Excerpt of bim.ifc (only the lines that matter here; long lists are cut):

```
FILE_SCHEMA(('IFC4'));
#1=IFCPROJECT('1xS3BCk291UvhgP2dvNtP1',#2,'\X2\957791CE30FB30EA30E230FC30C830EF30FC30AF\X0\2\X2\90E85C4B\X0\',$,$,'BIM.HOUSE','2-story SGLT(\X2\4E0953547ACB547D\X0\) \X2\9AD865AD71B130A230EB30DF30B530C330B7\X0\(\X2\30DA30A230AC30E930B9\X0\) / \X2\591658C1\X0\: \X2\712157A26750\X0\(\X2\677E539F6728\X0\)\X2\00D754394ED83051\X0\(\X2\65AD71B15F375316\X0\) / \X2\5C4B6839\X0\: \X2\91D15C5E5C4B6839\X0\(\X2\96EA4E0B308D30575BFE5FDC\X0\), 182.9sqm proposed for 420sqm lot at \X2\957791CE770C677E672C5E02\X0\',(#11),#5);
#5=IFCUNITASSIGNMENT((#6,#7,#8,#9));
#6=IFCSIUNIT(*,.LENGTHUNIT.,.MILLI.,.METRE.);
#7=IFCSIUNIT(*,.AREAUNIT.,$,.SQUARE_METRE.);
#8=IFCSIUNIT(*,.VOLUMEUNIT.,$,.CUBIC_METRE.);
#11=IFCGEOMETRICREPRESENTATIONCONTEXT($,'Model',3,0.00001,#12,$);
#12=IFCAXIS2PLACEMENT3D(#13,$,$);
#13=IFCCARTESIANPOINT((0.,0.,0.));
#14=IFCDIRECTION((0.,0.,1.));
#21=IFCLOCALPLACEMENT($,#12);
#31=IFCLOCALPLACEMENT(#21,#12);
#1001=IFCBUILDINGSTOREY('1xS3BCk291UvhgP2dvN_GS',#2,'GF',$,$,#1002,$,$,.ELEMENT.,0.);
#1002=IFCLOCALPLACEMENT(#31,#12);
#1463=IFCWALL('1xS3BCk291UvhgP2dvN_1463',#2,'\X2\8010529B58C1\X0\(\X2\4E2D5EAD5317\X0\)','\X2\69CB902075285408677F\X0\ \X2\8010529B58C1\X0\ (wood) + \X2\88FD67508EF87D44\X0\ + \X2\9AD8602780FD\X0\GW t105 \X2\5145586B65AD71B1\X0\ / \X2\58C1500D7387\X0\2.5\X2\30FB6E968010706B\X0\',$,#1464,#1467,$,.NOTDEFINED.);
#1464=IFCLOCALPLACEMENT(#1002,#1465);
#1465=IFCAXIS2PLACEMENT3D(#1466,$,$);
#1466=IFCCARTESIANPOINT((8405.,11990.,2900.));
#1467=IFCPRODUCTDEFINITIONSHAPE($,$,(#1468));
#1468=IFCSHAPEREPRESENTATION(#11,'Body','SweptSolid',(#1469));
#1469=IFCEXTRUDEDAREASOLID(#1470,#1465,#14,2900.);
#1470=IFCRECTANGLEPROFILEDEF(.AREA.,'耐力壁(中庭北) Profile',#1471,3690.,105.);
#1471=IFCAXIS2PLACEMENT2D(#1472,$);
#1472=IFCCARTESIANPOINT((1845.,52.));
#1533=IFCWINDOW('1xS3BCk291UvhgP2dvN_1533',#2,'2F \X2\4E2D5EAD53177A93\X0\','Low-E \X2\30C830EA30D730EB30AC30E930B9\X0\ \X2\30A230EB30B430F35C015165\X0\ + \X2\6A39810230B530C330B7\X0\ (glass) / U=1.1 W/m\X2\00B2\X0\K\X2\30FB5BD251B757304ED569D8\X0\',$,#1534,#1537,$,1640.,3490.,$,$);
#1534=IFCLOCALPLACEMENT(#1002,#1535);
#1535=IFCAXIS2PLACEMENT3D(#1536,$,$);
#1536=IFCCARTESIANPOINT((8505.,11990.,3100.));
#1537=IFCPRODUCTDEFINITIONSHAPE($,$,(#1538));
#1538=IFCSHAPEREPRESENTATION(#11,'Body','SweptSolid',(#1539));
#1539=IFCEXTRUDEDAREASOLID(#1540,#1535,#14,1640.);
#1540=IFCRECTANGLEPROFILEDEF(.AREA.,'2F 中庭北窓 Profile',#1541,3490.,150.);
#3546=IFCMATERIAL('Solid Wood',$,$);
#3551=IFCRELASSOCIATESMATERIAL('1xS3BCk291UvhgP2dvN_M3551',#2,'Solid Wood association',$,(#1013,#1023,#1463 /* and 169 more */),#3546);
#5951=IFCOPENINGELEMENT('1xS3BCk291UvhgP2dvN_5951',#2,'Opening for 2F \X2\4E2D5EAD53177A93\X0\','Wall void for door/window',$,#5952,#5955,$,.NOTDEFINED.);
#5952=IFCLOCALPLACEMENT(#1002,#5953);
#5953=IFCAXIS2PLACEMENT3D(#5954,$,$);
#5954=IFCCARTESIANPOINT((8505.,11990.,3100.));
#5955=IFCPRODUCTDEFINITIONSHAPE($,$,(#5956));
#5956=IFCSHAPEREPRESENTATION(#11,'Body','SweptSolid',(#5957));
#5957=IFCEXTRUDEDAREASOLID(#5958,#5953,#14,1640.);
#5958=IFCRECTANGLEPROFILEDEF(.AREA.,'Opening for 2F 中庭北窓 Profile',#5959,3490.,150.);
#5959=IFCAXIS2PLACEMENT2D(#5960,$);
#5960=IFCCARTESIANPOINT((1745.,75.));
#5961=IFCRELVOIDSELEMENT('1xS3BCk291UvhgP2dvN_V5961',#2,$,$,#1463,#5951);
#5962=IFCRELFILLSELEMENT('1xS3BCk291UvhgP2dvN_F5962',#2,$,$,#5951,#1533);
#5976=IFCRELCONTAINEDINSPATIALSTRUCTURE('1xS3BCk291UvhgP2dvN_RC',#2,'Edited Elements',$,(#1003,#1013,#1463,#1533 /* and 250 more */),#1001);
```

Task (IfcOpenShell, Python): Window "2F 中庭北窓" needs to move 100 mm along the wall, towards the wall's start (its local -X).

```python
import ifcopenshell
import ifcopenshell.api.geometry
import ifcopenshell.util.placement
import ifcopenshell.util.unit

model = ifcopenshell.open("bim.ifc")
unit_scale = ifcopenshell.util.unit.calculate_unit_scale(model)

window = model.by_guid("1xS3BCk291UvhgP2dvN_1533")
opening = window.FillsVoids[0].RelatingOpeningElement
wall = opening.VoidsElements[0].RelatingBuildingElement

wall_matrix = ifcopenshell.util.placement.get_local_placement(wall.ObjectPlacement)
shift = wall_matrix[:3, 0] * -0.1 / unit_scale
before = ifcopenshell.util.placement.get_local_placement(window.ObjectPlacement)[:3, 3].copy()

# The window is not placed relative to its opening, so move both.
for product in (opening, window):
    matrix = ifcopenshell.util.placement.get_local_placement(product.ObjectPlacement)
    matrix[:3, 3] += shift
    ifcopenshell.api.geometry.edit_object_placement(model, product=product, matrix=matrix, is_si=False)

after = ifcopenshell.util.placement.get_local_placement(window.ObjectPlacement)[:3, 3]
print("window moved by", (after - before).round(3) + 0.0)

model.write("bim_updated.ifc")
```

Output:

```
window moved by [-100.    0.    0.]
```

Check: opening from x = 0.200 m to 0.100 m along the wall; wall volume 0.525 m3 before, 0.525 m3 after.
